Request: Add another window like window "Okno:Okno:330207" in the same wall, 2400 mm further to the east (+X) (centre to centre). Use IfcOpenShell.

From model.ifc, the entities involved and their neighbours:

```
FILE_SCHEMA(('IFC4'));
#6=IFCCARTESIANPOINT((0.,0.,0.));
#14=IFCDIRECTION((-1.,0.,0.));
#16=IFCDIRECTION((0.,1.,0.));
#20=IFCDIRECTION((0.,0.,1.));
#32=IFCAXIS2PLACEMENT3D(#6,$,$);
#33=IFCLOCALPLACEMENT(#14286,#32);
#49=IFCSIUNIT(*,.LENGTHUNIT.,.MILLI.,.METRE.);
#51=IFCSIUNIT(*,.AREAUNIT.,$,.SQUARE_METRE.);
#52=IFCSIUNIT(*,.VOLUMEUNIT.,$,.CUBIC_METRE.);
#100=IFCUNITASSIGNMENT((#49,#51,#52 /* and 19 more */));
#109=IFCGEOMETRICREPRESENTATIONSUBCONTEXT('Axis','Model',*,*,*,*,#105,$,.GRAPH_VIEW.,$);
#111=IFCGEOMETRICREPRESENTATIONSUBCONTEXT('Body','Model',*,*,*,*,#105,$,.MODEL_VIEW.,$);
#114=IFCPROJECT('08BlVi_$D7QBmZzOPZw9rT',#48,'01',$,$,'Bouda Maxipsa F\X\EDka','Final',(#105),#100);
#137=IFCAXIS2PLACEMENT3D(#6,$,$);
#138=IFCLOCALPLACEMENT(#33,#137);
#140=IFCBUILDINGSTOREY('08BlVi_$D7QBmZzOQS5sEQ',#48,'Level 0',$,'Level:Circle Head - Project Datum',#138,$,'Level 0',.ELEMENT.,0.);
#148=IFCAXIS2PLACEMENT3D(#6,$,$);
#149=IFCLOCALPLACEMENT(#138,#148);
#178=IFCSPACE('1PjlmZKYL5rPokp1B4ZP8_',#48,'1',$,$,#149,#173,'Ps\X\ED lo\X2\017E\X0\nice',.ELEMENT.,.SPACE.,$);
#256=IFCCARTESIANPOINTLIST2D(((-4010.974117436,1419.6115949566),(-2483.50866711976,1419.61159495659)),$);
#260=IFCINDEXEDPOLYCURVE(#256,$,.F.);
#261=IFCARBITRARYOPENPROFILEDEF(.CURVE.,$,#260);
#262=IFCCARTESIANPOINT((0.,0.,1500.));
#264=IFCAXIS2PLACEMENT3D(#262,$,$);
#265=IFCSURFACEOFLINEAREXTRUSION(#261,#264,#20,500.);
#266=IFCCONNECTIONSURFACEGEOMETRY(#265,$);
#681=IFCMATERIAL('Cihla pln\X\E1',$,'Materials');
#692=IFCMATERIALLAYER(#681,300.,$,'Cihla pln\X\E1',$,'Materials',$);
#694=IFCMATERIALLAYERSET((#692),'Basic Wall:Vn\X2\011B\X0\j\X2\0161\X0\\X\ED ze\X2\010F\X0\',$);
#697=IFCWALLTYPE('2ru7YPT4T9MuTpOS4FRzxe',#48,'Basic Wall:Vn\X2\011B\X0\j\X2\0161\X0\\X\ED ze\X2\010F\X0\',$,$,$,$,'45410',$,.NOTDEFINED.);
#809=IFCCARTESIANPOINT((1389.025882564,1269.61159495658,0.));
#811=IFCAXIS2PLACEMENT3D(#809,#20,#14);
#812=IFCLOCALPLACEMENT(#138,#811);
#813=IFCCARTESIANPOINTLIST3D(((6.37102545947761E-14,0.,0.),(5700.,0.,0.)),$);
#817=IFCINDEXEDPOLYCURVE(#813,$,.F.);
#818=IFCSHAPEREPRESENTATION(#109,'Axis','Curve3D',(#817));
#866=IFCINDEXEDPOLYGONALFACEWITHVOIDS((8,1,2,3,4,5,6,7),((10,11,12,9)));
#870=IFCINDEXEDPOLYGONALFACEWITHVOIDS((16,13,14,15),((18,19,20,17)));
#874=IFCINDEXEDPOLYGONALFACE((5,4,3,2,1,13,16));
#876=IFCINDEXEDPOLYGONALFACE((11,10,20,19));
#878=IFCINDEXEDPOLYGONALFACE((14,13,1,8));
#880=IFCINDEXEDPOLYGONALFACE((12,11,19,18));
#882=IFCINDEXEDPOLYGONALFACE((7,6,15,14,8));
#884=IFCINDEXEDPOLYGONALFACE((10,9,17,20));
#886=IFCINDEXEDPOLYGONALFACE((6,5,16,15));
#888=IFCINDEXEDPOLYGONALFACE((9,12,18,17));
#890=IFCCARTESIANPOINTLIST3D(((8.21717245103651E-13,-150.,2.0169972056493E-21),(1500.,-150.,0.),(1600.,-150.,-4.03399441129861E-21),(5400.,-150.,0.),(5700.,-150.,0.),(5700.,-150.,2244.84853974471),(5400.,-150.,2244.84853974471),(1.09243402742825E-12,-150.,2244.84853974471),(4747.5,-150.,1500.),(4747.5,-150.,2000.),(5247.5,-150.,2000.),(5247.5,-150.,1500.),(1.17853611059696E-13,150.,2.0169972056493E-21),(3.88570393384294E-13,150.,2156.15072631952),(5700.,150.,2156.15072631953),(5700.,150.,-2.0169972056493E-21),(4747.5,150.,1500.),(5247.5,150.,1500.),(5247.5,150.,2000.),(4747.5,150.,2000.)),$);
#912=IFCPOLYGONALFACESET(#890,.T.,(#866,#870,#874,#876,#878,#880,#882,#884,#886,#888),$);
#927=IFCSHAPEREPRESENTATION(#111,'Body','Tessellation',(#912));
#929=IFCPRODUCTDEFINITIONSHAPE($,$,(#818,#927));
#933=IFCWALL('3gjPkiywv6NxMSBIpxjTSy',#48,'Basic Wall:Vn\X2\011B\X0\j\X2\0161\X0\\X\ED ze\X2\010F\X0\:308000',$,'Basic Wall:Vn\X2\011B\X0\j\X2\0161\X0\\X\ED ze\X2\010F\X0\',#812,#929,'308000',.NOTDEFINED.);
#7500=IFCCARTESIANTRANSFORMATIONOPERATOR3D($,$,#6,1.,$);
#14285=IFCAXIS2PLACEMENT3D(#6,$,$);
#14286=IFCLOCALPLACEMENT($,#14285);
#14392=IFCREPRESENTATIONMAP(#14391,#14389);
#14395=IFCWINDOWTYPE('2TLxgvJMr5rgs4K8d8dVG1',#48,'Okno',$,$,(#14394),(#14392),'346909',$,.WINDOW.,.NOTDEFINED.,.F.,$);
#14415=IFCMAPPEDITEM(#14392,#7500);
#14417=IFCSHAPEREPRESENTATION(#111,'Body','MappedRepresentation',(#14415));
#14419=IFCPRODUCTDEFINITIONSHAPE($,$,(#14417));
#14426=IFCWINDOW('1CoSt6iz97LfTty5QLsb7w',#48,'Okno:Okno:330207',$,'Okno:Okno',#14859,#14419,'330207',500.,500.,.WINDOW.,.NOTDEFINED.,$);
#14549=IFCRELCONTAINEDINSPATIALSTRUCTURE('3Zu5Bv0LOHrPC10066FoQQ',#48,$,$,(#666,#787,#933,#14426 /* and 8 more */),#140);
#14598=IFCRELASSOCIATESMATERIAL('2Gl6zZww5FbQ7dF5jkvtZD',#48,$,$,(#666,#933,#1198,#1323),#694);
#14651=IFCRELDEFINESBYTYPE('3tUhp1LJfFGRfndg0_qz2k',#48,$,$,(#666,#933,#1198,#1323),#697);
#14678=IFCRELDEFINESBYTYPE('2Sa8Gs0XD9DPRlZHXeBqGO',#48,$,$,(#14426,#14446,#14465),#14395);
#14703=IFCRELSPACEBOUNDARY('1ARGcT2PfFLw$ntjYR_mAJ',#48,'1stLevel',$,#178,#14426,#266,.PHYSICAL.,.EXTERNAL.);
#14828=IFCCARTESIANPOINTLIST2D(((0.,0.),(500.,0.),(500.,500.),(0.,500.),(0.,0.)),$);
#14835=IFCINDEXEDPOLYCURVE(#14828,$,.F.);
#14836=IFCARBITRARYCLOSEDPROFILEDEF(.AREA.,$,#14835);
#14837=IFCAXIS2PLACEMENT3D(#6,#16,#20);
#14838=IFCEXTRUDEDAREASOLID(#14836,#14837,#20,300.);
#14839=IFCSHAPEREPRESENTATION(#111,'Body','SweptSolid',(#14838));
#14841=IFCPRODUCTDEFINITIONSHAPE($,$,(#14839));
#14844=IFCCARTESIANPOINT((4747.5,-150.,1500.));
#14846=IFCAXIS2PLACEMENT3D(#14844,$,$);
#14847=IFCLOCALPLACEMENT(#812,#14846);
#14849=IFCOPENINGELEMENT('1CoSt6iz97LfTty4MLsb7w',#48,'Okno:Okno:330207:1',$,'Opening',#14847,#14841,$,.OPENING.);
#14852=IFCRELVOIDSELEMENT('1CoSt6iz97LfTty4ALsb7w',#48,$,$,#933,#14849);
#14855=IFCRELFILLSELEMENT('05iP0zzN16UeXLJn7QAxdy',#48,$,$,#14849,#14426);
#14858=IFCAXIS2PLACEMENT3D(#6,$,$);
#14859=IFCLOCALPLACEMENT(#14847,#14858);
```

```python
import numpy as np
import ifcopenshell
import ifcopenshell.api.feature
import ifcopenshell.api.geometry
import ifcopenshell.api.root
import ifcopenshell.geom
import ifcopenshell.util.element
import ifcopenshell.util.placement
import ifcopenshell.util.shape

model = ifcopenshell.open("model.ifc")
settings = ifcopenshell.geom.settings()


def volume(element):
    """Net volume in cubic metres, openings subtracted."""
    shape = ifcopenshell.geom.create_shape(settings, element)
    return ifcopenshell.util.shape.get_volume(shape.geometry)


window = model.by_guid("1CoSt6iz97LfTty5QLsb7w")
opening = window.FillsVoids[0].RelatingOpeningElement
wall = opening.VoidsElements[0].RelatingBuildingElement
before = volume(wall)
shift = ifcopenshell.util.placement.get_local_placement(wall.ObjectPlacement)[:3, 0] * -2400.0

# copy_class copies the void relationship, type, container and properties, but no geometry.
new_opening = ifcopenshell.api.root.copy_class(model, product=opening)
new_opening.Representation = ifcopenshell.util.element.copy_deep(
    model, opening.Representation, exclude=["IfcGeometricRepresentationContext", "IfcRepresentationMap"]
)
new_opening.Name = "Okno:Okno"
new_window = ifcopenshell.api.root.copy_class(model, product=window)
new_window.Representation = ifcopenshell.util.element.copy_deep(
    model, window.Representation, exclude=["IfcGeometricRepresentationContext", "IfcRepresentationMap"]
)
new_window.Name = "Okno:Okno"
new_window.Tag = None
ifcopenshell.api.feature.add_filling(model, opening=new_opening, element=new_window)

for old, new in ((opening, new_opening), (window, new_window)):
    matrix = ifcopenshell.util.placement.get_local_placement(old.ObjectPlacement)
    matrix[:3, 3] += shift
    ifcopenshell.api.geometry.edit_object_placement(model, product=new, matrix=matrix, is_si=False)

# The copied space boundaries still share their surfaces with the original.
for rel in new_window.ProvidesBoundaries:
    if rel.ConnectionGeometry:
        rel.ConnectionGeometry = ifcopenshell.util.element.copy_deep(model, rel.ConnectionGeometry)

# Space boundary surfaces are stored in each space's coordinates; move them too.
for rel in new_window.ProvidesBoundaries:
    if not rel.ConnectionGeometry:
        continue
    surface = rel.ConnectionGeometry.SurfaceOnRelatingElement
    space_matrix = ifcopenshell.util.placement.get_local_placement(rel.RelatingSpace.ObjectPlacement)
    point = np.array(surface.Position.Location.Coordinates) + space_matrix[:3, :3].T @ shift
    surface.Position = model.createIfcAxis2Placement3D(
        model.createIfcCartesianPoint(point.tolist()), surface.Position.Axis, surface.Position.RefDirection
    )

after = volume(wall)

print(f"wall volume {before:.3f} -> {after:.3f} m3")

model.write("model_rev.ifc")
```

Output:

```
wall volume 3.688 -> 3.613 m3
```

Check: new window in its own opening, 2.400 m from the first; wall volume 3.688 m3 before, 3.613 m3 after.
